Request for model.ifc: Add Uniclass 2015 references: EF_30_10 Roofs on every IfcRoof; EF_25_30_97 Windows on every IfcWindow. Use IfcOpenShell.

First a look at what the model holds.

```python
import ifcopenshell

model = ifcopenshell.open("model.ifc")
print(model.schema)
print("classifications:", [c.Name for c in model.by_type("IfcClassification")])
for ifc_class in ("IfcDoor", "IfcRoof", "IfcStair", "IfcWall", "IfcWindow"):
    print(ifc_class, len(model.by_type(ifc_class)))
```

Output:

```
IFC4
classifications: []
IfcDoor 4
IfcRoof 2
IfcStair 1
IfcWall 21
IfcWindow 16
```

```python
import ifcopenshell
import ifcopenshell.api.classification

model = ifcopenshell.open("model.ifc")

system = ifcopenshell.api.classification.add_classification(model, classification="Uniclass 2015")

codes = {
    "IfcRoof": ("EF_30_10", "Roofs"),
    "IfcWindow": ("EF_25_30_97", "Windows"),
}
for ifc_class, (code, name) in codes.items():
    products = model.by_type(ifc_class)
    ifcopenshell.api.classification.add_reference(
        model, products=products, classification=system, identification=code, name=name
    )
    print(code, len(products))

model.write("model_updated.ifc")
```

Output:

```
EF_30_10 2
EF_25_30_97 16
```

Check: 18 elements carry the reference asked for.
